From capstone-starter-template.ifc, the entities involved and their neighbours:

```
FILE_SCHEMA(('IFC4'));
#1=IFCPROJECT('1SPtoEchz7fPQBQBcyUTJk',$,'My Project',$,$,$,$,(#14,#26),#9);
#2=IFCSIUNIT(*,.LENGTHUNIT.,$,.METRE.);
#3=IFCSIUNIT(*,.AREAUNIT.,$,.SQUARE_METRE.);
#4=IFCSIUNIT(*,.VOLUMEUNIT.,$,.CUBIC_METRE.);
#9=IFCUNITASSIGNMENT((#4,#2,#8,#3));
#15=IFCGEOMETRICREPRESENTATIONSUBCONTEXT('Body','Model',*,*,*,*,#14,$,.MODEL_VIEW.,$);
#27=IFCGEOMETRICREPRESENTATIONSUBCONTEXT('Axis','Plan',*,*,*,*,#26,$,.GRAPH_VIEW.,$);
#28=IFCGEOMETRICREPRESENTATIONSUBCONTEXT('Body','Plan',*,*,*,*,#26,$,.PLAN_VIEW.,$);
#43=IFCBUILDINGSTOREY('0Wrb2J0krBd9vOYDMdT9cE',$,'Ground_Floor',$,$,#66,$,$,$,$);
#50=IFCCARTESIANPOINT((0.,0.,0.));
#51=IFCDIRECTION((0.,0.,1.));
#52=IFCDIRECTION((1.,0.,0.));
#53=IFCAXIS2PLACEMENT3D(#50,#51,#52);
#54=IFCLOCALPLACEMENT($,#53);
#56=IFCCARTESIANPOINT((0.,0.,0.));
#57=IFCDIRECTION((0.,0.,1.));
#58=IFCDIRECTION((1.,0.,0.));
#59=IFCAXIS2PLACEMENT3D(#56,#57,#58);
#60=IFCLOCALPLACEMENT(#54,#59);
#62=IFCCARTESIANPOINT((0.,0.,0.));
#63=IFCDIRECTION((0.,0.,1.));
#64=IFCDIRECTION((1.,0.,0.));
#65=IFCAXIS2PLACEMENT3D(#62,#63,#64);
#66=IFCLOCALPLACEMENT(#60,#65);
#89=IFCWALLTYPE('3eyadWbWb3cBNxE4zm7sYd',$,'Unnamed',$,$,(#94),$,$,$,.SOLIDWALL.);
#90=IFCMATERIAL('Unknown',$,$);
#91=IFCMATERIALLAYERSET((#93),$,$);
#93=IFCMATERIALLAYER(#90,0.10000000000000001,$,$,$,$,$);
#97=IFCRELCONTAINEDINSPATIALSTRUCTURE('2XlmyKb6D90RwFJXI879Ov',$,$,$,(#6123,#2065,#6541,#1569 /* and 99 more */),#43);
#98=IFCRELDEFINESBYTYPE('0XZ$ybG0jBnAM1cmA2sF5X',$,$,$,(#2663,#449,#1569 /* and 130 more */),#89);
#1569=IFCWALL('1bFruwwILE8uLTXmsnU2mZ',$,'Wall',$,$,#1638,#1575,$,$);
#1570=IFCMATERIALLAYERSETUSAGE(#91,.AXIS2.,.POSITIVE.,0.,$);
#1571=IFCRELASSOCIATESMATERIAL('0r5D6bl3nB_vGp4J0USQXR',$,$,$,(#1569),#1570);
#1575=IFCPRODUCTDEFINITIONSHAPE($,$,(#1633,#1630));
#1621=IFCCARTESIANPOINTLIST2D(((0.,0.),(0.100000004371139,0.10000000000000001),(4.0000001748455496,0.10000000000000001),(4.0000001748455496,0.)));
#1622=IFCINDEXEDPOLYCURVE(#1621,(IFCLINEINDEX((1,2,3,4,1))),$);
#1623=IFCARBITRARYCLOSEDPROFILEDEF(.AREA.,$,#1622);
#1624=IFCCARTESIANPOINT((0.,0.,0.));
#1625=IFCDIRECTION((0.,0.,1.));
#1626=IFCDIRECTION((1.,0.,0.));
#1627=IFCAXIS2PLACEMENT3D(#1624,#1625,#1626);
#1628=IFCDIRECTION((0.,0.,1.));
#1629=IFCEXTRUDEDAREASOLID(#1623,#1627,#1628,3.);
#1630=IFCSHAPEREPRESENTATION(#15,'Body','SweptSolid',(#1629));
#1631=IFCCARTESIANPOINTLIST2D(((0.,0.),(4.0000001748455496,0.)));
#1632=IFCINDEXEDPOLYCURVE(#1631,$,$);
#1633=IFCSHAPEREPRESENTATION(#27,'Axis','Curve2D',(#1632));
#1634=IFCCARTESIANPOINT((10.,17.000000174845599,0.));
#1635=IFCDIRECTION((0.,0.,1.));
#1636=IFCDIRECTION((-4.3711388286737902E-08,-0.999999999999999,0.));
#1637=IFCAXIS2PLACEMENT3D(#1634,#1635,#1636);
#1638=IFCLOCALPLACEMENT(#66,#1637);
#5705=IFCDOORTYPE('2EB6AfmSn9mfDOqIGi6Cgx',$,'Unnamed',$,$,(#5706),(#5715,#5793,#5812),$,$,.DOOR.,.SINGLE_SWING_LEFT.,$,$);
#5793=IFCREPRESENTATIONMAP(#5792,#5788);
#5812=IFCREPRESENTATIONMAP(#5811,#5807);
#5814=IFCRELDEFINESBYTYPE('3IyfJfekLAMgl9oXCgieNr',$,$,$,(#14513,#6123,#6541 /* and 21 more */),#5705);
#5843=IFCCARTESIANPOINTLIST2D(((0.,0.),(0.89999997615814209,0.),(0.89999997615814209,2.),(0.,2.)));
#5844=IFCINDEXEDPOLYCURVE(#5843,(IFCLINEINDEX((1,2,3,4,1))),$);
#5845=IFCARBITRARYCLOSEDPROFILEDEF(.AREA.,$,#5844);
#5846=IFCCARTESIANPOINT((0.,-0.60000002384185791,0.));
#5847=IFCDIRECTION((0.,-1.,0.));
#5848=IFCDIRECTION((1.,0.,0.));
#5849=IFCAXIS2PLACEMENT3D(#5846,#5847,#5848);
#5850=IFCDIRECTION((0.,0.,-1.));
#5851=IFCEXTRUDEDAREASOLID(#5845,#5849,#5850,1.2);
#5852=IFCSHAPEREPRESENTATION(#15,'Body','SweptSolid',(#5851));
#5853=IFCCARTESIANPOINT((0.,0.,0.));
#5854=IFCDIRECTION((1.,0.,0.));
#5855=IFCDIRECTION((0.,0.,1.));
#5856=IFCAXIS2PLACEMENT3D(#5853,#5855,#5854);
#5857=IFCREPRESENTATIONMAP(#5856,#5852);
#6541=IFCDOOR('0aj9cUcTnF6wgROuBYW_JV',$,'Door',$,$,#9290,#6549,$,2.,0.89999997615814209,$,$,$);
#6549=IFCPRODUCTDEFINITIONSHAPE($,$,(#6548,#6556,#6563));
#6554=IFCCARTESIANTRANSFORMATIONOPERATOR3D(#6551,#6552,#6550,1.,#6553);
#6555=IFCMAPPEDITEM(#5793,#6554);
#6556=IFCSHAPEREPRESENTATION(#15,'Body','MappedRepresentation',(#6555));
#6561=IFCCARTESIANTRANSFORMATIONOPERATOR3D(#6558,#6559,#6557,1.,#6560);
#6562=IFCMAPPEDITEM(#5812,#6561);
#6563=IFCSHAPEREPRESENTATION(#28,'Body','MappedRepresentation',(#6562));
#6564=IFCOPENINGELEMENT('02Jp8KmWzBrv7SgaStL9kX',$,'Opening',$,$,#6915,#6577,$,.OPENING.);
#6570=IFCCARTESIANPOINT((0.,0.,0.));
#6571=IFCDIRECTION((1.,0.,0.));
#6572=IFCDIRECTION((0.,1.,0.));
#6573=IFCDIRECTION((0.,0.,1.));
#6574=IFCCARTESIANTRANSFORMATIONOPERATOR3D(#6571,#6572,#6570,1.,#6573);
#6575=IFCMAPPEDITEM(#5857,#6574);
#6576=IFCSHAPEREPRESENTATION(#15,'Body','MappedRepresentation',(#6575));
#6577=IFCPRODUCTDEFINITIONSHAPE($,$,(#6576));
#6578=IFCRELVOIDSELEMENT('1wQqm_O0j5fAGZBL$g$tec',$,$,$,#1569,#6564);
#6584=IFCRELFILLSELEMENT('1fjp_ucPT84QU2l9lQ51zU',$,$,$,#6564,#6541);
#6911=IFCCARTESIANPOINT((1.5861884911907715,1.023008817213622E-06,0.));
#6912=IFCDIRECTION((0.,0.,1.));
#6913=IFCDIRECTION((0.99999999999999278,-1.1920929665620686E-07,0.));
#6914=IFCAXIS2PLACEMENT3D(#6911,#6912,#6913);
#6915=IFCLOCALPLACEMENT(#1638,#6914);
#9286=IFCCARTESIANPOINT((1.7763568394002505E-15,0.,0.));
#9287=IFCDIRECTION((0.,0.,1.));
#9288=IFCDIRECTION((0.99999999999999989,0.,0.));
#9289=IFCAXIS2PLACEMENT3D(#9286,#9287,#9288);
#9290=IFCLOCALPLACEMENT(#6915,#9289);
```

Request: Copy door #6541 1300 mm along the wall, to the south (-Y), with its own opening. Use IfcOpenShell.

```python
import ifcopenshell
import ifcopenshell.api.feature
import ifcopenshell.api.geometry
import ifcopenshell.api.root
import ifcopenshell.geom
import ifcopenshell.util.element
import ifcopenshell.util.placement
import ifcopenshell.util.shape
import ifcopenshell.util.unit

model = ifcopenshell.open("capstone-starter-template.ifc")
unit_scale = ifcopenshell.util.unit.calculate_unit_scale(model)
settings = ifcopenshell.geom.settings()


def volume(element):
    """Net volume in cubic metres, openings subtracted."""
    shape = ifcopenshell.geom.create_shape(settings, element)
    return ifcopenshell.util.shape.get_volume(shape.geometry)


door = model.by_guid("0aj9cUcTnF6wgROuBYW_JV")
opening = door.FillsVoids[0].RelatingOpeningElement
wall = opening.VoidsElements[0].RelatingBuildingElement
before = volume(wall)
shift = ifcopenshell.util.placement.get_local_placement(wall.ObjectPlacement)[:3, 0] * 1.3 / unit_scale

# copy_class copies the void relationship, type, container and properties, but no geometry.
new_opening = ifcopenshell.api.root.copy_class(model, product=opening)
new_opening.Representation = ifcopenshell.util.element.copy_deep(
    model, opening.Representation, exclude=["IfcGeometricRepresentationContext", "IfcRepresentationMap"]
)
new_door = ifcopenshell.api.root.copy_class(model, product=door)
new_door.Representation = ifcopenshell.util.element.copy_deep(
    model, door.Representation, exclude=["IfcGeometricRepresentationContext", "IfcRepresentationMap"]
)
ifcopenshell.api.feature.add_filling(model, opening=new_opening, element=new_door)

for old, new in ((opening, new_opening), (door, new_door)):
    matrix = ifcopenshell.util.placement.get_local_placement(old.ObjectPlacement)
    matrix[:3, 3] += shift
    ifcopenshell.api.geometry.edit_object_placement(model, product=new, matrix=matrix, is_si=False)

after = volume(wall)

print(f"wall volume {before:.3f} -> {after:.3f} m3")

model.write("capstone-starter-template_updated.ifc")
```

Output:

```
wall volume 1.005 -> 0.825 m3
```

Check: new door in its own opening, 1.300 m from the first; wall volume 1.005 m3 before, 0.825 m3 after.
